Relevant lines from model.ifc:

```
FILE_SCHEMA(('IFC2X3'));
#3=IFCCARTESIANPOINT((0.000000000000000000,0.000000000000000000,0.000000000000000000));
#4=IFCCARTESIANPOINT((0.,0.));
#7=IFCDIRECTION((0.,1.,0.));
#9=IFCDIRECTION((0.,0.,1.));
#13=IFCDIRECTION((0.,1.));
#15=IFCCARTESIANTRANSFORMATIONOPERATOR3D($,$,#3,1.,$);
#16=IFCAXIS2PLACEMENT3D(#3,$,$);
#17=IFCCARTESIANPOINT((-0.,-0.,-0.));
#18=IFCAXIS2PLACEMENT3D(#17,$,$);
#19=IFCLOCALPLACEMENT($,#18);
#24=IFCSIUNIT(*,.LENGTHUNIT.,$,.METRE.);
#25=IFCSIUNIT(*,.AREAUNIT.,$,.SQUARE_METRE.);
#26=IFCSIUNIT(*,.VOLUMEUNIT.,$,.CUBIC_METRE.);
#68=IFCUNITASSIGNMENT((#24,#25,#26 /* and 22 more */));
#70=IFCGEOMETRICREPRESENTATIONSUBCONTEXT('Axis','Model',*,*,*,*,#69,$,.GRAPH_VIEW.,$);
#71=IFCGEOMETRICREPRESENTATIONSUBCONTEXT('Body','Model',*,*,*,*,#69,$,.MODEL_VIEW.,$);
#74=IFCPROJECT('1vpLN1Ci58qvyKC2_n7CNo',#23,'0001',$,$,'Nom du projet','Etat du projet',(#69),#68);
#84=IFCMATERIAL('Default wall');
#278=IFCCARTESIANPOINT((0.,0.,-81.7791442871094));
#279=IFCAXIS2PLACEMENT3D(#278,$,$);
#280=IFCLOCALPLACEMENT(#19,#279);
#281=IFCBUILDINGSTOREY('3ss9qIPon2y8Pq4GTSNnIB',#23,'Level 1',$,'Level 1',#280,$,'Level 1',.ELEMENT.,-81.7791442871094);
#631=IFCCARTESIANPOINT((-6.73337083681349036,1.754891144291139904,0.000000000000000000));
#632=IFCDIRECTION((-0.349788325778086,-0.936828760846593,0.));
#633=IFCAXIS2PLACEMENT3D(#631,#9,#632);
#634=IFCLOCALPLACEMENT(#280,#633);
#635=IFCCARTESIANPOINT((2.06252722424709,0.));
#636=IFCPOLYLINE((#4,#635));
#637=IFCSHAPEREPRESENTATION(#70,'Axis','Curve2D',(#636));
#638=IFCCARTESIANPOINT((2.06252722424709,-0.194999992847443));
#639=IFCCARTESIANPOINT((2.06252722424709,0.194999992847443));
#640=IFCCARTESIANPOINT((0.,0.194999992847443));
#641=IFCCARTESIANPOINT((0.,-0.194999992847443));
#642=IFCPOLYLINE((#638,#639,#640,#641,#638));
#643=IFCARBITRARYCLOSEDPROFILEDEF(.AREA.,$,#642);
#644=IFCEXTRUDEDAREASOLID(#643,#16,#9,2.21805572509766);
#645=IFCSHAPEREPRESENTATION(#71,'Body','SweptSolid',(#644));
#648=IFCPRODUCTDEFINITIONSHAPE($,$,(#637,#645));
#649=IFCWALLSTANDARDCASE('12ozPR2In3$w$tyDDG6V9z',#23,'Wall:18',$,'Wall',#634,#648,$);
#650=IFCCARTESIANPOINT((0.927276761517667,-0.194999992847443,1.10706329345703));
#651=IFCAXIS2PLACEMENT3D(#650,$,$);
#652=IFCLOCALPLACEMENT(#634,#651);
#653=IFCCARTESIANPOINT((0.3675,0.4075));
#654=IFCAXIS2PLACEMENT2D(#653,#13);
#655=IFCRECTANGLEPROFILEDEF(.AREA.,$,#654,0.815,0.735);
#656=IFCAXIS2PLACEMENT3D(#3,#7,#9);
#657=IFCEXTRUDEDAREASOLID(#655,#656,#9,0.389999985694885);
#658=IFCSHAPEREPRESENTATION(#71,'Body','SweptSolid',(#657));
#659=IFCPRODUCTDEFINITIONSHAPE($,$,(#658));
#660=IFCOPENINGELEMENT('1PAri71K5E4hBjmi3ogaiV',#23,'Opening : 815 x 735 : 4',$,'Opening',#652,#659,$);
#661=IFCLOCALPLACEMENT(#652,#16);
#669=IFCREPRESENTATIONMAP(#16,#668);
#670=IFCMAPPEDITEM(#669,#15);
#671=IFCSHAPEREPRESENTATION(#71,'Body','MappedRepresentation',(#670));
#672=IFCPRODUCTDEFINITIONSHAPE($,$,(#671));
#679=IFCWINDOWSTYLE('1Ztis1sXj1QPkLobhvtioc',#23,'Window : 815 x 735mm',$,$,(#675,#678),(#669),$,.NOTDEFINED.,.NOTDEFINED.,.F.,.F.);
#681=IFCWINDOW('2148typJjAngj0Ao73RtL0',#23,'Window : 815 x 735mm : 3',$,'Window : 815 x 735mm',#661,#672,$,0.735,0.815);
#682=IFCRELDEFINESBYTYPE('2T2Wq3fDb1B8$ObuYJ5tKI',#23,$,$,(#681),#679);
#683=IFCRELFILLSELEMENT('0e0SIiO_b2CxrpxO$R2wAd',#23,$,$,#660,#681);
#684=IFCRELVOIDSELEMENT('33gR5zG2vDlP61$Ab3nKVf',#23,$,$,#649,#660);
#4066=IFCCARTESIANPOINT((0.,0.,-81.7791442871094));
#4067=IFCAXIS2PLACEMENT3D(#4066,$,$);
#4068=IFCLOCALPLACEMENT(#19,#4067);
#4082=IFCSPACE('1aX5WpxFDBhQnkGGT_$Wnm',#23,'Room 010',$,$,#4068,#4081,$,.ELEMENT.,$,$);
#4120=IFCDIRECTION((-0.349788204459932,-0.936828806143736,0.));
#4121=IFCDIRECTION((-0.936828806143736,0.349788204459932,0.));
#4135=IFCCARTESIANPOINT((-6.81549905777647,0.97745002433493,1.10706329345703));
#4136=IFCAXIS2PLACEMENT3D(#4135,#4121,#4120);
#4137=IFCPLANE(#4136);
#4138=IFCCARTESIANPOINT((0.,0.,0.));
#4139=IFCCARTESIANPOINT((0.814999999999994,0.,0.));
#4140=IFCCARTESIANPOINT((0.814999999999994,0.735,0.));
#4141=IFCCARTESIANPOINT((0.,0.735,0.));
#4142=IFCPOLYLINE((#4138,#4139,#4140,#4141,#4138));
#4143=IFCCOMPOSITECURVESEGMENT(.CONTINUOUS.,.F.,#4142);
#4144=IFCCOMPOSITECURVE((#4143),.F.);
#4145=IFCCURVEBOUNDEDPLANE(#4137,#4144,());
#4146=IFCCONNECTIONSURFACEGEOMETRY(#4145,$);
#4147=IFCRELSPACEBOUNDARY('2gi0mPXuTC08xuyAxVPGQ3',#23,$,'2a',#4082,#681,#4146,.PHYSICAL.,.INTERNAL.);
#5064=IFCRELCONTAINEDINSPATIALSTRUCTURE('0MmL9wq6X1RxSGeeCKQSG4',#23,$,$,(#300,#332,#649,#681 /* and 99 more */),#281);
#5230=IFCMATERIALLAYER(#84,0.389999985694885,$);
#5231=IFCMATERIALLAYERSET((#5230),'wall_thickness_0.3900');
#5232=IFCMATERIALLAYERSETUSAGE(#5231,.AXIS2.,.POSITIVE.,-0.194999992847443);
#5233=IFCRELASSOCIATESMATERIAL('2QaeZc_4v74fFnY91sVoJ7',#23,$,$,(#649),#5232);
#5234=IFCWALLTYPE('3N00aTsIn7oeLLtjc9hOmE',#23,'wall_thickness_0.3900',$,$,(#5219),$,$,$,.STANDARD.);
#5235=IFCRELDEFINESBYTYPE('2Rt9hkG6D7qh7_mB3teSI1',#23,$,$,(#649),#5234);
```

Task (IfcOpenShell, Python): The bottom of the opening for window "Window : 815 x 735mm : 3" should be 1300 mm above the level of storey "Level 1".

```python
import numpy as np
import ifcopenshell
import ifcopenshell.api.geometry
import ifcopenshell.geom
import ifcopenshell.util.element
import ifcopenshell.util.placement
import ifcopenshell.util.shape
import ifcopenshell.util.unit

model = ifcopenshell.open("model.ifc")
unit_scale = ifcopenshell.util.unit.calculate_unit_scale(model)

window = model.by_guid("2148typJjAngj0Ao73RtL0")
opening = window.FillsVoids[0].RelatingOpeningElement
storey = ifcopenshell.util.element.get_container(window, ifc_class="IfcBuildingStorey")
level = ifcopenshell.util.placement.get_local_placement(storey.ObjectPlacement)[2, 3]

# The opening's origin need not be at the sill, so measure its lowest point.
shape = ifcopenshell.geom.create_shape(ifcopenshell.geom.settings(), opening)
bottom = ifcopenshell.util.shape.get_shape_bottom_elevation(shape, shape.geometry) / unit_scale
dz = level + 1.3 - bottom

shift = np.array([0.0, 0.0, dz])
# The window is placed relative to its opening, so it follows when the opening moves.
matrix = ifcopenshell.util.placement.get_local_placement(opening.ObjectPlacement)
matrix[:3, 3] += shift
ifcopenshell.api.geometry.edit_object_placement(
    model, product=opening, matrix=matrix, is_si=False, should_transform_children=True
)

# Space boundary surfaces are stored in each space's coordinates; move them too.
for rel in window.ProvidesBoundaries:
    if not rel.ConnectionGeometry:
        continue
    surface = rel.ConnectionGeometry.SurfaceOnRelatingElement.BasisSurface
    space_matrix = ifcopenshell.util.placement.get_local_placement(rel.RelatingSpace.ObjectPlacement)
    point = np.array(surface.Position.Location.Coordinates) + space_matrix[:3, :3].T @ shift
    surface.Position = model.createIfcAxis2Placement3D(
        model.createIfcCartesianPoint(point.tolist()), surface.Position.Axis, surface.Position.RefDirection
    )

print(f"moved by {dz * unit_scale:+.3f} m")

model.write("model-out.ifc")
```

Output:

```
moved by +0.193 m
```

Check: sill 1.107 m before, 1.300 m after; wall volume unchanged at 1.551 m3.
